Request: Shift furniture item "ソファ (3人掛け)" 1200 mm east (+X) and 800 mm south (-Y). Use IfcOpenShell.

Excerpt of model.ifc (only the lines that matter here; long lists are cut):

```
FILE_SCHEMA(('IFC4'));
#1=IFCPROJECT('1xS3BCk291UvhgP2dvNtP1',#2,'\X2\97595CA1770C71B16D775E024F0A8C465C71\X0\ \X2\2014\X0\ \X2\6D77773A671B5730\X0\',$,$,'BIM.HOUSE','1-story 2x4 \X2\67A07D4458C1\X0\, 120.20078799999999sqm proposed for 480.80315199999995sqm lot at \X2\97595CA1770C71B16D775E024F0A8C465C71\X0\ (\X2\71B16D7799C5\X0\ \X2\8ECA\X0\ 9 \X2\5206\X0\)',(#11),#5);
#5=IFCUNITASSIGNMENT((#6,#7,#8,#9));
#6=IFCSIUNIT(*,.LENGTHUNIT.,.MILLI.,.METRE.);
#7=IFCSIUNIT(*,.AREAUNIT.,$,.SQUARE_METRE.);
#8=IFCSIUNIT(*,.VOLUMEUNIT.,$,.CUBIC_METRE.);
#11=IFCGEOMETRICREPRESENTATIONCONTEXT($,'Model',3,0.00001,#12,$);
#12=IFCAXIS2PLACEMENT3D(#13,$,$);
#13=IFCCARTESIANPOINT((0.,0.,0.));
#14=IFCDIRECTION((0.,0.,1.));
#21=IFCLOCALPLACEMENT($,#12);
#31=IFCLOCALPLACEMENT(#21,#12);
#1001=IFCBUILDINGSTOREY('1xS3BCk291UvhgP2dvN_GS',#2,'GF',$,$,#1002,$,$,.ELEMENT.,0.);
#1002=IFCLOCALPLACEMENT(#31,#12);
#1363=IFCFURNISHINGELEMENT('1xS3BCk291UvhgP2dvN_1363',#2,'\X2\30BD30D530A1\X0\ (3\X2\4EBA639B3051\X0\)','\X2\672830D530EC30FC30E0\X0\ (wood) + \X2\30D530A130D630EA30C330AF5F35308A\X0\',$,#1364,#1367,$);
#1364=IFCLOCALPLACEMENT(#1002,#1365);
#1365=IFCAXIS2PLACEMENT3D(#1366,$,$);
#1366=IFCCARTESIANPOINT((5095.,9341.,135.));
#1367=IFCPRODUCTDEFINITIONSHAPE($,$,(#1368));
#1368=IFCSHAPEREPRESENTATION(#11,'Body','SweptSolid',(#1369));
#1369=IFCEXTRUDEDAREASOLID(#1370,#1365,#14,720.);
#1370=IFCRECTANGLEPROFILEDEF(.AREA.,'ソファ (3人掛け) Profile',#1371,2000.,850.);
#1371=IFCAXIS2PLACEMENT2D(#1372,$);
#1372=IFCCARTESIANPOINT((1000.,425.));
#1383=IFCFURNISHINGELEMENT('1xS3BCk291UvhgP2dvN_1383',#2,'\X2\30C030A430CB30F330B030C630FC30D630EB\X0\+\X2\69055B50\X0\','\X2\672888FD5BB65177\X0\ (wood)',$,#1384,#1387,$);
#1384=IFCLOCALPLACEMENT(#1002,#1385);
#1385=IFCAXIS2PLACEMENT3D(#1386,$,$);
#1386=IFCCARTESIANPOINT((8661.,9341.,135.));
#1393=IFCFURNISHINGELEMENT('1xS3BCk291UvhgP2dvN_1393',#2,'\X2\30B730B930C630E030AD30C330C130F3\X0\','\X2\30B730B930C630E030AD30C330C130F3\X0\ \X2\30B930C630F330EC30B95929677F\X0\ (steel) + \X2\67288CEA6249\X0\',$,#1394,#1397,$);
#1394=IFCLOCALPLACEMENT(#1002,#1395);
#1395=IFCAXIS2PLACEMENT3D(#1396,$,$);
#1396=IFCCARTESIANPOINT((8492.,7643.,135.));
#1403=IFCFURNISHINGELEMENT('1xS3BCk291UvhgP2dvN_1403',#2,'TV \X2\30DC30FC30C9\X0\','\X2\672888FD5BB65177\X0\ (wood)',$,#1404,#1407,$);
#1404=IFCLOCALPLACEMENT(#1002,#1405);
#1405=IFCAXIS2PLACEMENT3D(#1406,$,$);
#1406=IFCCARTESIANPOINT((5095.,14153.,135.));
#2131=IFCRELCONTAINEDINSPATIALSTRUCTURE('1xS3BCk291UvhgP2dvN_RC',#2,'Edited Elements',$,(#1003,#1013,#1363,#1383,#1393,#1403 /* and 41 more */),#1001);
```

```python
import ifcopenshell
import ifcopenshell.api.geometry
import ifcopenshell.util.placement

model = ifcopenshell.open("model.ifc")

item = model.by_guid("1xS3BCk291UvhgP2dvN_1363")
matrix = ifcopenshell.util.placement.get_local_placement(item.ObjectPlacement)
matrix[0, 3] += 1200.0
matrix[1, 3] -= 800.0
ifcopenshell.api.geometry.edit_object_placement(model, product=item, matrix=matrix, is_si=False)

print(ifcopenshell.util.placement.get_local_placement(item.ObjectPlacement).round(3) + 0.0)

model.write("model_v2.ifc")
```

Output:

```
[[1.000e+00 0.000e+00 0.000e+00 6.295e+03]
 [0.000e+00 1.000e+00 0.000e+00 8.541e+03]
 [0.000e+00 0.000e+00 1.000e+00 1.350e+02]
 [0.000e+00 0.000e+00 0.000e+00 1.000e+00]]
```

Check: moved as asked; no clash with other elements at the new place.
